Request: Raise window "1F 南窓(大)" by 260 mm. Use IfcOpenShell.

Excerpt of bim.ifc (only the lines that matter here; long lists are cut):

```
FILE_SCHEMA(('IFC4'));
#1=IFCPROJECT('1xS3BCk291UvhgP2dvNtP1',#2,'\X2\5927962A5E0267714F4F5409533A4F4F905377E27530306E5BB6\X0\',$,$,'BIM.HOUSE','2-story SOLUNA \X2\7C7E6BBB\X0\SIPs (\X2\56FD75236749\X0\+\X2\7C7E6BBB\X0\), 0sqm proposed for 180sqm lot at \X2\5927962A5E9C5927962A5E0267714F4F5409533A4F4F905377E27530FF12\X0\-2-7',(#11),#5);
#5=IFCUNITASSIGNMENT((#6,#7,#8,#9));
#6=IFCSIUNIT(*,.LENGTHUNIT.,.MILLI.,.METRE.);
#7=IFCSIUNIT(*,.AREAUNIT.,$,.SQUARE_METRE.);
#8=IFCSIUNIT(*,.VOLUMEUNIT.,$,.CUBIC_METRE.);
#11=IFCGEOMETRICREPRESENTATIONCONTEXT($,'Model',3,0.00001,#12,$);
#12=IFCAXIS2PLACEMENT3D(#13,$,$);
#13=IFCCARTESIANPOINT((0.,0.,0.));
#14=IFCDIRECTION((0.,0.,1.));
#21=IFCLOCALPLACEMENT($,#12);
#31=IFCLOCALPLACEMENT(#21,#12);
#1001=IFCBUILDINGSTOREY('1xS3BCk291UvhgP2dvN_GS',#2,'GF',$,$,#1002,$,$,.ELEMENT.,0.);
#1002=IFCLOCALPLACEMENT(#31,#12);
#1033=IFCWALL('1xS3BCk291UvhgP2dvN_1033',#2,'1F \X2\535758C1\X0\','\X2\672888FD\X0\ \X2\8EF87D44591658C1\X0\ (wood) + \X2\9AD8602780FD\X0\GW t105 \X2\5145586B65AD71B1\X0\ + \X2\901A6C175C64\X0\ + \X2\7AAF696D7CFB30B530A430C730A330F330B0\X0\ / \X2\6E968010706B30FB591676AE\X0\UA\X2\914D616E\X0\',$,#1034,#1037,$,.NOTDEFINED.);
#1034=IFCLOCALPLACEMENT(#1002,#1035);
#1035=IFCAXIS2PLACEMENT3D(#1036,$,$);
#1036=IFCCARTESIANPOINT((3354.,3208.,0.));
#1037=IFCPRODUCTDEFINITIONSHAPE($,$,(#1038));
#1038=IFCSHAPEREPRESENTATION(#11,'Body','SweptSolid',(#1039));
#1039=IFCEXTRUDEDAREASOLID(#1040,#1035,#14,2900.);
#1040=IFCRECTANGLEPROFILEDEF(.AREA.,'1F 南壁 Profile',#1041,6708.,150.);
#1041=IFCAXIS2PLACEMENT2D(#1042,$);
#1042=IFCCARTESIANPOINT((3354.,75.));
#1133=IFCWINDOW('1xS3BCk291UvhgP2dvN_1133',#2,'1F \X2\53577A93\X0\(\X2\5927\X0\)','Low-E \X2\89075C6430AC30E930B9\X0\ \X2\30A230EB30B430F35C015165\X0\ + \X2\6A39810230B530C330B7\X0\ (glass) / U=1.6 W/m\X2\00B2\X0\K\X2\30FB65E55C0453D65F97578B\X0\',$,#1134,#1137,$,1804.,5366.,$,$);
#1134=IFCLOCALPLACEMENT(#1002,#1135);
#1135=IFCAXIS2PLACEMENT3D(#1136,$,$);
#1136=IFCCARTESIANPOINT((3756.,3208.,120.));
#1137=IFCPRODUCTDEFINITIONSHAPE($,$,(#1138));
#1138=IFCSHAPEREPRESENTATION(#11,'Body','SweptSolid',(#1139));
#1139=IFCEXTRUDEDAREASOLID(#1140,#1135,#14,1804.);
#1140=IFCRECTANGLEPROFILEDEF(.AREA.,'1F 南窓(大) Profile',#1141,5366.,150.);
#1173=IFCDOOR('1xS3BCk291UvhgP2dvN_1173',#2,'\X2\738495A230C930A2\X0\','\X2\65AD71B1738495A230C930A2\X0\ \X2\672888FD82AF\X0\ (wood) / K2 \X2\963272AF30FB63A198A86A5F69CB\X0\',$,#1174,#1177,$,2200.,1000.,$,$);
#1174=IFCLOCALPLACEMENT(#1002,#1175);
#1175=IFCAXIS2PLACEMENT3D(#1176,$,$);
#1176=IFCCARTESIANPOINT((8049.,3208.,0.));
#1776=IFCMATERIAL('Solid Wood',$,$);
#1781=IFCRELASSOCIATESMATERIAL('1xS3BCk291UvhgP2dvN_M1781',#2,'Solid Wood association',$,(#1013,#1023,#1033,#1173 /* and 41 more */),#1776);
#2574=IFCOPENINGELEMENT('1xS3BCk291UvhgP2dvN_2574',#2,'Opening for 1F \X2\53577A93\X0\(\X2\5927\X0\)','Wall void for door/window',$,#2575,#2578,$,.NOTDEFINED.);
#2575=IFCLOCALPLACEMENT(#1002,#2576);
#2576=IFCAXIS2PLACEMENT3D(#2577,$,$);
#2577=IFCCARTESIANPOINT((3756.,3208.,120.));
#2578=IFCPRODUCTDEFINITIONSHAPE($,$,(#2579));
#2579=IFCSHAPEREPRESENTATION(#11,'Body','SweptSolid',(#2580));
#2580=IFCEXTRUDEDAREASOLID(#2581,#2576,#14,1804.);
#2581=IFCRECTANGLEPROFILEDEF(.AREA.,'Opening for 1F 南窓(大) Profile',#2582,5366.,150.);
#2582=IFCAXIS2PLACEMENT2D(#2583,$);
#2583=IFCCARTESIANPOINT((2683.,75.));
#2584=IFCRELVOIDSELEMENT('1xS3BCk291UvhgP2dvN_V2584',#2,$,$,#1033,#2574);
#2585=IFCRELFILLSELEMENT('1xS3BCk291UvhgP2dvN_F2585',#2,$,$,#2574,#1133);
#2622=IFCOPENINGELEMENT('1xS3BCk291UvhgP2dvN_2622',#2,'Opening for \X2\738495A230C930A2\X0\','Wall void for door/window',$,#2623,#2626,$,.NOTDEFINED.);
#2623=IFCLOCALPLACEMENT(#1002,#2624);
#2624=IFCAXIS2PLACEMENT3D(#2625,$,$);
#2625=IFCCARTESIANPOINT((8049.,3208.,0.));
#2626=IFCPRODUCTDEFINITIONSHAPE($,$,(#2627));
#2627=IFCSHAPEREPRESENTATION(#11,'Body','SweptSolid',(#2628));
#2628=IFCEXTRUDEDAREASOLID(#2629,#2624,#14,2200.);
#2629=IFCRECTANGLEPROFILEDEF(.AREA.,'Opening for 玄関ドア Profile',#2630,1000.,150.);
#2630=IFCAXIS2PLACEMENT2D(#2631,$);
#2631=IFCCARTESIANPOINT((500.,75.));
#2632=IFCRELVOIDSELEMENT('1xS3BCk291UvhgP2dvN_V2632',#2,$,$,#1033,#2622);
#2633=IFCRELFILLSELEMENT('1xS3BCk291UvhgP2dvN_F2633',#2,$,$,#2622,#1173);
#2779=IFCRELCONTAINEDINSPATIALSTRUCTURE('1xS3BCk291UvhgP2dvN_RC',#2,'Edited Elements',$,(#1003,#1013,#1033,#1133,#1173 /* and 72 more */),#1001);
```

```python
import numpy as np
import ifcopenshell
import ifcopenshell.api.geometry
import ifcopenshell.util.placement
import ifcopenshell.util.unit

model = ifcopenshell.open("bim.ifc")
unit_scale = ifcopenshell.util.unit.calculate_unit_scale(model)

window = model.by_guid("1xS3BCk291UvhgP2dvN_1133")
opening = window.FillsVoids[0].RelatingOpeningElement
dz = 260.0

shift = np.array([0.0, 0.0, dz])
# The window is not placed relative to its opening, so move both.
for product in (opening, window):
    matrix = ifcopenshell.util.placement.get_local_placement(product.ObjectPlacement)
    matrix[:3, 3] += shift
    ifcopenshell.api.geometry.edit_object_placement(model, product=product, matrix=matrix, is_si=False)

print(f"moved by {dz * unit_scale:+.3f} m")

model.write("bim_updated.ifc")
```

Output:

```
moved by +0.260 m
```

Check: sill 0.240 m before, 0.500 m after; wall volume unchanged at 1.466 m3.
